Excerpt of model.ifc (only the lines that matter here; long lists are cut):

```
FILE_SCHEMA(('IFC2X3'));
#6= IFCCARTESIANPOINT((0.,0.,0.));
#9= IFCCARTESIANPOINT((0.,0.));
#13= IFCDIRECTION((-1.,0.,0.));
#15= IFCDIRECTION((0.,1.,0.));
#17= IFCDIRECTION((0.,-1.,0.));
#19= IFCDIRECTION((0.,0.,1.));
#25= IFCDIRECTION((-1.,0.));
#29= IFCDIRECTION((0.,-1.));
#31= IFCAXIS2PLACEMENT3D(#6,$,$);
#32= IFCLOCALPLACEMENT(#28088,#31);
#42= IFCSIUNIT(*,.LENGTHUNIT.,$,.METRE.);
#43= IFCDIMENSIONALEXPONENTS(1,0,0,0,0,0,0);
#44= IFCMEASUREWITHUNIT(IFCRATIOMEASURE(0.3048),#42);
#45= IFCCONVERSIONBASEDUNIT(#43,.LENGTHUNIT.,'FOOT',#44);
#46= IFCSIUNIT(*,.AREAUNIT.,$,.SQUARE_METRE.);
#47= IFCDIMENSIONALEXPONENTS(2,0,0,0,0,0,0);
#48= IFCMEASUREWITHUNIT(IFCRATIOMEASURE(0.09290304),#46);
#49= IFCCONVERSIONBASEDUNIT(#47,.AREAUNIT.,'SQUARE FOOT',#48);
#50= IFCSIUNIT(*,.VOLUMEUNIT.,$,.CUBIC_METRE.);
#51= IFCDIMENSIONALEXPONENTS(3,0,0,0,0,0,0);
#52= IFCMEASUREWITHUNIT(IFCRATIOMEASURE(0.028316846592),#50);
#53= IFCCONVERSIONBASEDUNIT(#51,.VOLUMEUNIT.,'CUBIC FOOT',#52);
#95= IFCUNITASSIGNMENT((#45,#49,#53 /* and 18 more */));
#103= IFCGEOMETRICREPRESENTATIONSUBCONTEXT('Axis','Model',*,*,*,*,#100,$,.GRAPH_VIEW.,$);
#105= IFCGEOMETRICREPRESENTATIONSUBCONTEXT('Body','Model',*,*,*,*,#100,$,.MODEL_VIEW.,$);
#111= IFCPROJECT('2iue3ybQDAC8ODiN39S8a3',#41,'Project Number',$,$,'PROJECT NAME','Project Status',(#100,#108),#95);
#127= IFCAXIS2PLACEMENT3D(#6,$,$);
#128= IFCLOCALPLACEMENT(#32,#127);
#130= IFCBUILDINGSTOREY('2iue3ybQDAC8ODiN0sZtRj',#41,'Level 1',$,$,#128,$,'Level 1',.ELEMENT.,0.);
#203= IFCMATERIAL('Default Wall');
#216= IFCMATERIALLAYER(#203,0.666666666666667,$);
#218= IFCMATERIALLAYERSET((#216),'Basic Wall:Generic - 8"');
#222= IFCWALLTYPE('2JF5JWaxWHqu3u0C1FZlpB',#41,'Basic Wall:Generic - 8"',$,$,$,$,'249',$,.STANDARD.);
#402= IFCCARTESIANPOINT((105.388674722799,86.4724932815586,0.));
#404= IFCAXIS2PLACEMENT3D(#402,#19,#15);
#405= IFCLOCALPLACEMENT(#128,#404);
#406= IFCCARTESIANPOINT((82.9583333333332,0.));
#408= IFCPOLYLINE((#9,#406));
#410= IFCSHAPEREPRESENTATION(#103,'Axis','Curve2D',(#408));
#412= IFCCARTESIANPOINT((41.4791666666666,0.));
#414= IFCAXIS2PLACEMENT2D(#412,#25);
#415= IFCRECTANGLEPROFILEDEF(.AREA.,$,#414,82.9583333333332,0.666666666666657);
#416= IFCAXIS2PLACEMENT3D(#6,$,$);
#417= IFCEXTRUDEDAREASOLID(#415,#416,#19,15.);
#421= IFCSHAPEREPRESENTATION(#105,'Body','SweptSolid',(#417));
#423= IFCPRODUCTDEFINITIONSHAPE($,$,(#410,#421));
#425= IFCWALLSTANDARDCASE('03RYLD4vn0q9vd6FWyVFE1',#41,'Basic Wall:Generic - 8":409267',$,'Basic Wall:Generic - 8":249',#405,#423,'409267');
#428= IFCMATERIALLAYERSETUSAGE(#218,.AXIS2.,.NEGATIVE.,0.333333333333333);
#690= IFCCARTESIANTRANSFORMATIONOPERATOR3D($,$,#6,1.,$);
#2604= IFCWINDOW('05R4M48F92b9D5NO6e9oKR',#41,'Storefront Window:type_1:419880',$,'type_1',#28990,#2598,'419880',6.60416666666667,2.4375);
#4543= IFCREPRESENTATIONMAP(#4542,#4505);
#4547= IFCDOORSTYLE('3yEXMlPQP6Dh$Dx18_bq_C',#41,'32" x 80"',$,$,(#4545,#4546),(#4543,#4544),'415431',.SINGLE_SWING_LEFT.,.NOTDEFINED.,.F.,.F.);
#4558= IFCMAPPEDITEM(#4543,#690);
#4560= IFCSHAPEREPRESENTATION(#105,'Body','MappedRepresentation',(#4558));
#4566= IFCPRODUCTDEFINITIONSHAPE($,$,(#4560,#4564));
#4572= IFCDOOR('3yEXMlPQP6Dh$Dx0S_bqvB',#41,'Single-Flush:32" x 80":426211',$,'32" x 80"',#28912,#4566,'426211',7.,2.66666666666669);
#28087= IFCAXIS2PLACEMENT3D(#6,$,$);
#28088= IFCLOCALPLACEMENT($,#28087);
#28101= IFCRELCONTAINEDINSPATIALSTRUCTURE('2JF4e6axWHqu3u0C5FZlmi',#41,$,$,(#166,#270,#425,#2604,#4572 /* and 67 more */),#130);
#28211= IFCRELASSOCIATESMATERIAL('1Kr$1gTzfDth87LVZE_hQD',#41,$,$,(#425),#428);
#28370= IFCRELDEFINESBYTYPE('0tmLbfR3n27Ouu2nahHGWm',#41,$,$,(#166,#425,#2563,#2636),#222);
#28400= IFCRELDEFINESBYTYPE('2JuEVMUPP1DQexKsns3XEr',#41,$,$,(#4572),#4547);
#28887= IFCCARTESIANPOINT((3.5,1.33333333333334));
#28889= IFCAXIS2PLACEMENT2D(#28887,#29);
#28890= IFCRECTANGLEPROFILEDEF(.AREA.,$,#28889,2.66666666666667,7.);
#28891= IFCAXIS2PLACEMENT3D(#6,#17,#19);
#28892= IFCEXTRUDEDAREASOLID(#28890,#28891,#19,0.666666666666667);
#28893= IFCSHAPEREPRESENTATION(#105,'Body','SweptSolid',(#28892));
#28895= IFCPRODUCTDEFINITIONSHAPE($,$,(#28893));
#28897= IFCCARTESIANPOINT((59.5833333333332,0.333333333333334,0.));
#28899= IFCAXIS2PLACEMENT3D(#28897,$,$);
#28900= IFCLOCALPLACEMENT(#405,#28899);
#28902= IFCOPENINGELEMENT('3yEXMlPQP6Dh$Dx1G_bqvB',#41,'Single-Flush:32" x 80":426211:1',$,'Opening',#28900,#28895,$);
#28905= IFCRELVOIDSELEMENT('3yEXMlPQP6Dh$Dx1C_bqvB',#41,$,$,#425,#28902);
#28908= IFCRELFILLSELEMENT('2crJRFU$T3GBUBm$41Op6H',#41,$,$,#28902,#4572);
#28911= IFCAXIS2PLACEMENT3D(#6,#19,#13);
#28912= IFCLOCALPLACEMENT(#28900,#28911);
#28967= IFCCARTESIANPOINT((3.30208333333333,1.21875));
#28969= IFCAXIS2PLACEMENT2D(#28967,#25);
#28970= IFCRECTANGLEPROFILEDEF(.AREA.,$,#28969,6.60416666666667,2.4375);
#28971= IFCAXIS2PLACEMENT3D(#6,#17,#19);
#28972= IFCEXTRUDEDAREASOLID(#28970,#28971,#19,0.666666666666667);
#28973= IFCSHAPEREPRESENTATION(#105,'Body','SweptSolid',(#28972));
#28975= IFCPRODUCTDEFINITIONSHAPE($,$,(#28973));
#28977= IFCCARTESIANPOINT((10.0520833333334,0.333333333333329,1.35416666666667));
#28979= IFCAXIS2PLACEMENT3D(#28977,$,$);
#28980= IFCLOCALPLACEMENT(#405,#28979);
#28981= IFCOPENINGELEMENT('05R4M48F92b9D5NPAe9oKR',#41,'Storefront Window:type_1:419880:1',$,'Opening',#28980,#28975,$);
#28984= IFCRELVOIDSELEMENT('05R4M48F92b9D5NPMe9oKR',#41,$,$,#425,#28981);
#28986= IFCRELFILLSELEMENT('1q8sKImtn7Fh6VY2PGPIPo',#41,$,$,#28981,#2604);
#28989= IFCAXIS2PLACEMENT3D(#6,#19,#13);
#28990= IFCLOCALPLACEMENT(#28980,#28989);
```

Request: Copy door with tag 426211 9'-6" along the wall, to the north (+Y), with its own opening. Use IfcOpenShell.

```python
import ifcopenshell
import ifcopenshell.api.feature
import ifcopenshell.api.geometry
import ifcopenshell.api.root
import ifcopenshell.geom
import ifcopenshell.util.element
import ifcopenshell.util.placement
import ifcopenshell.util.shape
import ifcopenshell.util.unit

model = ifcopenshell.open("model.ifc")
unit_scale = ifcopenshell.util.unit.calculate_unit_scale(model)
settings = ifcopenshell.geom.settings()


def volume(element):
    """Net volume in cubic metres, openings subtracted."""
    shape = ifcopenshell.geom.create_shape(settings, element)
    return ifcopenshell.util.shape.get_volume(shape.geometry)


def reuse_history(source, copy):
    """copy_class also copies each property set's owner history, people and application; keep the originals."""
    for rel in copy.IsDefinedBy:
        if rel.is_a("IfcRelDefinesByProperties") and (history := rel.RelatingPropertyDefinition.OwnerHistory):
            rel.RelatingPropertyDefinition.OwnerHistory = source.OwnerHistory
            ifcopenshell.util.element.remove_deep2(model, history)


door = model.by_guid("3yEXMlPQP6Dh$Dx0S_bqvB")
opening = door.FillsVoids[0].RelatingOpeningElement
wall = opening.VoidsElements[0].RelatingBuildingElement
before = volume(wall)
shift = ifcopenshell.util.placement.get_local_placement(wall.ObjectPlacement)[:3, 0] * 114 * 0.0254 / unit_scale

# copy_class copies the void relationship, type, container and properties, but no geometry.
new_opening = ifcopenshell.api.root.copy_class(model, product=opening)
new_opening.Representation = ifcopenshell.util.element.copy_deep(
    model, opening.Representation, exclude=["IfcGeometricRepresentationContext", "IfcRepresentationMap"]
)
new_opening.Name = 'Single-Flush:32" x 80"'
new_door = ifcopenshell.api.root.copy_class(model, product=door)
new_door.Representation = ifcopenshell.util.element.copy_deep(
    model, door.Representation, exclude=["IfcGeometricRepresentationContext", "IfcRepresentationMap"]
)
new_door.Name = 'Single-Flush:32" x 80"'
new_door.Tag = None
reuse_history(door, new_door)
fills = ifcopenshell.api.feature.add_filling(model, opening=new_opening, element=new_door)
fills.OwnerHistory = new_door.OwnerHistory  # required in IFC2X3

for old, new in ((opening, new_opening), (door, new_door)):
    matrix = ifcopenshell.util.placement.get_local_placement(old.ObjectPlacement)
    matrix[:3, 3] += shift
    ifcopenshell.api.geometry.edit_object_placement(model, product=new, matrix=matrix, is_si=False)

after = volume(wall)

print(f"wall volume {before:.3f} -> {after:.3f} m3")

model.write("model_edited.ifc")
```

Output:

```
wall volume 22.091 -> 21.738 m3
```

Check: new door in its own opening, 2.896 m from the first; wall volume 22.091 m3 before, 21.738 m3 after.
